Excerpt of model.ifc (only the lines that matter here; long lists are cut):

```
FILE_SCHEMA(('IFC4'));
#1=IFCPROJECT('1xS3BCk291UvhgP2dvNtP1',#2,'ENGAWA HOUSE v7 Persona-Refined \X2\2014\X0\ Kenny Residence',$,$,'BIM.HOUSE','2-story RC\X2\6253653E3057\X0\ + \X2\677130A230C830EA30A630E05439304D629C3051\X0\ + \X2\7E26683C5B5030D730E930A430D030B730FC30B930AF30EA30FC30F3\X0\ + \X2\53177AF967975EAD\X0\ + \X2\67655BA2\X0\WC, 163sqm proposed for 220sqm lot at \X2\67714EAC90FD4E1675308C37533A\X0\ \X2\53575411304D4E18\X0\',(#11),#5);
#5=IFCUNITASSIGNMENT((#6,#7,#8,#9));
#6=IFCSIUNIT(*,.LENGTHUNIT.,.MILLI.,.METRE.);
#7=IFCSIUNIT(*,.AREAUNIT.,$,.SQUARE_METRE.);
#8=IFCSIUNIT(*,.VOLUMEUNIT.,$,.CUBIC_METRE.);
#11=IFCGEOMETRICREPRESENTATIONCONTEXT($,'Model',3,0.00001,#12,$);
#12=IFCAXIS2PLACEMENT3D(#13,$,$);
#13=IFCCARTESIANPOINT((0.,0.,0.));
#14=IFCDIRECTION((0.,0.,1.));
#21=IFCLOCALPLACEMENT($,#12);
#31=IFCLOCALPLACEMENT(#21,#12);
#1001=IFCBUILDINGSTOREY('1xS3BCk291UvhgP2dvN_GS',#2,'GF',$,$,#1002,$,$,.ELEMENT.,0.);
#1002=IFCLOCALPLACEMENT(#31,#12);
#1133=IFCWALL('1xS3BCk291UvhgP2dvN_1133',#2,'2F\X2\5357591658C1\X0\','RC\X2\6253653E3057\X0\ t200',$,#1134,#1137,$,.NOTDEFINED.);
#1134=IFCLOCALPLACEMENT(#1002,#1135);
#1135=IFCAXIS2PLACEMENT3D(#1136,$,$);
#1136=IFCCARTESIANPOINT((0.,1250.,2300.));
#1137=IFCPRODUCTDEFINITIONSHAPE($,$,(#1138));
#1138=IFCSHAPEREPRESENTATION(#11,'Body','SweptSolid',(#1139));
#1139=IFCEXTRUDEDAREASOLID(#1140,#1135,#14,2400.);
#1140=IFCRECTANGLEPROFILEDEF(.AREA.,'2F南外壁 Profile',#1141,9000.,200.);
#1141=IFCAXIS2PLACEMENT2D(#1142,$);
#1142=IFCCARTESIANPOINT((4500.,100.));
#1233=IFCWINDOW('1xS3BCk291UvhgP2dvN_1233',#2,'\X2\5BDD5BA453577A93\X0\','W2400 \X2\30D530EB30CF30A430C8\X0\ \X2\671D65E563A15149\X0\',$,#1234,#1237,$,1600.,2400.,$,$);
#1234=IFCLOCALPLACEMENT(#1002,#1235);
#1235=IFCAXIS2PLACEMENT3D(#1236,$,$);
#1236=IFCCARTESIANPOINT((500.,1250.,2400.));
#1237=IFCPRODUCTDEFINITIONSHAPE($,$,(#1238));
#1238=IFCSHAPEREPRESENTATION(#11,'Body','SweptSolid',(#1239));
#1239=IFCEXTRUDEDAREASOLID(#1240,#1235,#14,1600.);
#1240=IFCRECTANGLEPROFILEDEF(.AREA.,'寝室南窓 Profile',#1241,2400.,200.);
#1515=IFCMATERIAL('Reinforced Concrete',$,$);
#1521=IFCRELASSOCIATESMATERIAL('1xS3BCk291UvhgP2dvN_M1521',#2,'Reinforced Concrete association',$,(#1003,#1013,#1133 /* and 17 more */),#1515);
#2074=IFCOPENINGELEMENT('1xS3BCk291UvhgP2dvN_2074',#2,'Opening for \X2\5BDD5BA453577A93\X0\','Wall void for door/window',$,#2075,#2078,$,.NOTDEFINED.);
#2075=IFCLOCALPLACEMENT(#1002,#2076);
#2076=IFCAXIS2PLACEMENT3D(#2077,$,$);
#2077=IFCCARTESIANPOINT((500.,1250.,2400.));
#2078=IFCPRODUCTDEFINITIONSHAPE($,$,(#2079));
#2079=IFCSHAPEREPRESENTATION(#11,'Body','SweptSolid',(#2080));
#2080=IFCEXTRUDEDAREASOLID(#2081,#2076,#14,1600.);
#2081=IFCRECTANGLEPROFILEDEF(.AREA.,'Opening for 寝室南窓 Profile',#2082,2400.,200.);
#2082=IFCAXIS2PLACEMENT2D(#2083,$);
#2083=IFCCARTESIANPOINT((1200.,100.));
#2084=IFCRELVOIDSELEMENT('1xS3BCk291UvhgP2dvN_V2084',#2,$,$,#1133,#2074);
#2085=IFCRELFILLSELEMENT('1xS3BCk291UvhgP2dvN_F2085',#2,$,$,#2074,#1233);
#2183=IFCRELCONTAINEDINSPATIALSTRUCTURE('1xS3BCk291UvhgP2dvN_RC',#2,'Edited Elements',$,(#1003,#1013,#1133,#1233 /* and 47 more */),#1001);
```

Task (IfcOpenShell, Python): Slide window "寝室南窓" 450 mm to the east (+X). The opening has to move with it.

```python
import ifcopenshell
import ifcopenshell.api.geometry
import ifcopenshell.util.placement
import ifcopenshell.util.unit

model = ifcopenshell.open("model.ifc")
unit_scale = ifcopenshell.util.unit.calculate_unit_scale(model)

window = model.by_id(1233)
opening = window.FillsVoids[0].RelatingOpeningElement
wall = opening.VoidsElements[0].RelatingBuildingElement

wall_matrix = ifcopenshell.util.placement.get_local_placement(wall.ObjectPlacement)
shift = wall_matrix[:3, 0] * 0.45 / unit_scale
before = ifcopenshell.util.placement.get_local_placement(window.ObjectPlacement)[:3, 3].copy()

# The window is not placed relative to its opening, so move both.
for product in (opening, window):
    matrix = ifcopenshell.util.placement.get_local_placement(product.ObjectPlacement)
    matrix[:3, 3] += shift
    ifcopenshell.api.geometry.edit_object_placement(model, product=product, matrix=matrix, is_si=False)

after = ifcopenshell.util.placement.get_local_placement(window.ObjectPlacement)[:3, 3]
print("window moved by", (after - before).round(3) + 0.0)

model.write("model_edited.ifc")
```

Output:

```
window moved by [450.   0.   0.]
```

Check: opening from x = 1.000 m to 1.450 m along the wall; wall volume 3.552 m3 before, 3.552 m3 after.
